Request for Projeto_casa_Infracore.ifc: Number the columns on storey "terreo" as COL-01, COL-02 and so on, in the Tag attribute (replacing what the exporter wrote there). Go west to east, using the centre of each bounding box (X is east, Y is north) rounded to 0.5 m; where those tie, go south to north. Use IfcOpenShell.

First a look at what the model holds.

```python
import ifcopenshell
import ifcopenshell.util.element
import ifcopenshell.util.placement

model = ifcopenshell.open("Projeto_casa_Infracore.ifc")
print(model.schema)
storey = next(s for s in model.by_type("IfcBuildingStorey") if s.Name == "terreo")
columns = [e for e in ifcopenshell.util.element.get_decomposition(storey) if e.is_a("IfcColumn")]
for e in sorted(columns, key=lambda e: e.id()):
    origin = ifcopenshell.util.placement.get_local_placement(e.ObjectPlacement)[:3, 3]
    print(e.id(), e.Tag, e.Name, origin.round(2) + 0.0, sep=" | ")
```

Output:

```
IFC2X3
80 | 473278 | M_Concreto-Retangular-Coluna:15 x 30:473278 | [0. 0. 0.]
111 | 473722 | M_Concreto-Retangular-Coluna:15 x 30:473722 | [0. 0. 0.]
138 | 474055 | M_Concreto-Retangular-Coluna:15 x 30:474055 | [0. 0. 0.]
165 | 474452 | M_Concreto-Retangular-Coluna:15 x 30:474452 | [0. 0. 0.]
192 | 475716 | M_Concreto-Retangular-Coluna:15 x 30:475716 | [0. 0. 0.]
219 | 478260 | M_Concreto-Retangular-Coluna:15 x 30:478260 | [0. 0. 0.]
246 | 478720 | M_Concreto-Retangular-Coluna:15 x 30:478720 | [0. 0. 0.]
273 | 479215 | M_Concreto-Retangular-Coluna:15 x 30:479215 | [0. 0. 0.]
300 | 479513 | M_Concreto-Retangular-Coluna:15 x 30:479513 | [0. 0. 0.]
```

```python
import ifcopenshell
import ifcopenshell.geom
import ifcopenshell.util.element
import ifcopenshell.util.shape

model = ifcopenshell.open("Projeto_casa_Infracore.ifc")
settings = ifcopenshell.geom.settings()
settings.set("use-world-coords", True)


def centre(element):
    shape = ifcopenshell.geom.create_shape(settings, element)
    return ifcopenshell.util.shape.get_bbox_centroid(shape.geometry)


storey = next(s for s in model.by_type("IfcBuildingStorey") if s.Name == "terreo")
columns = [e for e in ifcopenshell.util.element.get_decomposition(storey) if e.is_a("IfcColumn")]

# Insertion points can sit at a corner or the storey origin, so sort by the geometry (in metres).
centres = {e: centre(e) for e in columns}
columns.sort(key=lambda e: (round(centres[e][0] / 0.5), centres[e][1]))

for i, e in enumerate(columns, start=1):
    number = f"COL-{i:02d}"
    e.Tag = number
    print(e.id(), number)

model.write("Projeto_casa_Infracore_edited.ifc")
```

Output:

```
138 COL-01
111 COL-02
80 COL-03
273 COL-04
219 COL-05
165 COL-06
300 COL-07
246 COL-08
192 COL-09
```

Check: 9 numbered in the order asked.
